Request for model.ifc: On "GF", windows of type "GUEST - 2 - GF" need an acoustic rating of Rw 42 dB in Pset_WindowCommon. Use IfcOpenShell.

First a look at what the model holds.

```python
import ifcopenshell
import ifcopenshell.util.element

model = ifcopenshell.open("model.ifc")
print(model.schema)
storey = next(s for s in model.by_type("IfcBuildingStorey") if s.Name == "GF")
windows = [e for e in ifcopenshell.util.element.get_decomposition(storey) if e.is_a("IfcWindow")]
seen = {}
for e in windows:
    element_type = ifcopenshell.util.element.get_type(e)
    key = (element_type.Name if element_type != e and element_type else None, ifcopenshell.util.element.get_pset(e, "Pset_WindowCommon", "AcousticRating"))
    seen[key] = seen.get(key, 0) + 1
for (name, value), count in sorted(seen.items(), key=str):
    print(count, "x", name, "|", value)
```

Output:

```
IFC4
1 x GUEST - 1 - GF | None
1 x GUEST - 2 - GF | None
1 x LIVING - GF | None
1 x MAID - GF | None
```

```python
import ifcopenshell
import ifcopenshell.api.pset
import ifcopenshell.util.element

model = ifcopenshell.open("model.ifc")

storey = next(s for s in model.by_type("IfcBuildingStorey") if s.Name == "GF")
windows = [e for e in ifcopenshell.util.element.get_decomposition(storey) if e.is_a("IfcWindow")]

count = 0
for e in windows:
    element_type = ifcopenshell.util.element.get_type(e)
    if element_type in (None, e) or element_type.Name != "GUEST - 2 - GF":
        continue
    # add_pset returns the element's existing set when there is one.
    pset = ifcopenshell.api.pset.add_pset(model, product=e, name="Pset_WindowCommon")
    ifcopenshell.api.pset.edit_pset(model, pset=pset, properties={"AcousticRating": "Rw 42 dB"})
    count += 1

print(count, "windows updated")

model.write("model_edited.ifc")
```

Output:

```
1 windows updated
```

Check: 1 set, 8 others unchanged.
